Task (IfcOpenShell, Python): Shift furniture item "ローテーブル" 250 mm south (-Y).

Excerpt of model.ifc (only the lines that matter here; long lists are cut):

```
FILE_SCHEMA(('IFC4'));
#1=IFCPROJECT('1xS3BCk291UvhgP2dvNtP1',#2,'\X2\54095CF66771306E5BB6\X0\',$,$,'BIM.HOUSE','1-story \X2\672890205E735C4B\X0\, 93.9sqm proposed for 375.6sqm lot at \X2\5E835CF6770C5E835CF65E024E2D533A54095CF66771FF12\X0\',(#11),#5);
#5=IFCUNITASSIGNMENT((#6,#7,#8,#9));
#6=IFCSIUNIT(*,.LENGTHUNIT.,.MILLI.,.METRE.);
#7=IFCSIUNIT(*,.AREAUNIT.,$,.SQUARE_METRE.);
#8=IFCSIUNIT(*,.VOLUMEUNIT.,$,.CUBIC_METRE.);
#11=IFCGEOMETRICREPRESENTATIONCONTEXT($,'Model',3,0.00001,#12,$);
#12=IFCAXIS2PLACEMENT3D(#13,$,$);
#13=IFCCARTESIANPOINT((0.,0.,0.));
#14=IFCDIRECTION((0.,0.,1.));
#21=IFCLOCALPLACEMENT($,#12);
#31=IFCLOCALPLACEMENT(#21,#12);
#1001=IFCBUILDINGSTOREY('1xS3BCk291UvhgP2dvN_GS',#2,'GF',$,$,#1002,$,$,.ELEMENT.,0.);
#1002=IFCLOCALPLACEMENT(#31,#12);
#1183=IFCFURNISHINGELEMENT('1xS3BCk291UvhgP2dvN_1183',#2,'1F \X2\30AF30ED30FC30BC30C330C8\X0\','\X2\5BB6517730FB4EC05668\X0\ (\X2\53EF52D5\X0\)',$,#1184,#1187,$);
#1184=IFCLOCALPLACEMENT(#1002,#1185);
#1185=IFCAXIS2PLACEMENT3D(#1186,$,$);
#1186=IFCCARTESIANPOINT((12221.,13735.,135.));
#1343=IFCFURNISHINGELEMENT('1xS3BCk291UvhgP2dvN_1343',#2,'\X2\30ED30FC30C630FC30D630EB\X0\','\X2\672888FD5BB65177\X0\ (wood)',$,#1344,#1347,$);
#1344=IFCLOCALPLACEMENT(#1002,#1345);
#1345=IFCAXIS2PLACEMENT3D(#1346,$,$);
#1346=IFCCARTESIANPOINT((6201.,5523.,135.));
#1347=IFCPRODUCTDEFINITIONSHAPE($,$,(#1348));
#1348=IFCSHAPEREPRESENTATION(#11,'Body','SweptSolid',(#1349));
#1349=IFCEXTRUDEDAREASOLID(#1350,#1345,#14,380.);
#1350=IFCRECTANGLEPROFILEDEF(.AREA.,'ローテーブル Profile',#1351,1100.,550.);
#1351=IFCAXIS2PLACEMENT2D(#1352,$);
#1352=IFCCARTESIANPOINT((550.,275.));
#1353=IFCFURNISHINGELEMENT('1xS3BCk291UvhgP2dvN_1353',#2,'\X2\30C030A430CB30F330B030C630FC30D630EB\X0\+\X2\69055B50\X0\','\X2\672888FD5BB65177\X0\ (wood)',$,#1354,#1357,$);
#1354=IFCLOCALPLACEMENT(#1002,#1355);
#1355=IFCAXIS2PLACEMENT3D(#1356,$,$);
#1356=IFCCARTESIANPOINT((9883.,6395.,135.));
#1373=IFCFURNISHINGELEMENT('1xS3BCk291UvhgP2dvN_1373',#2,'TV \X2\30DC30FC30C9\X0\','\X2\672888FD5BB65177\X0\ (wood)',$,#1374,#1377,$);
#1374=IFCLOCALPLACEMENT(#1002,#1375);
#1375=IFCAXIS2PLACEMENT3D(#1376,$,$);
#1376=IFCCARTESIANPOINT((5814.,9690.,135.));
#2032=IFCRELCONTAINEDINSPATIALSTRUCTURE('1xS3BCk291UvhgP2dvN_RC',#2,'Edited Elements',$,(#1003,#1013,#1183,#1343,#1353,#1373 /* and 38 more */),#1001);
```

```python
import ifcopenshell
import ifcopenshell.api.geometry
import ifcopenshell.util.placement

model = ifcopenshell.open("model.ifc")

item = model.by_guid("1xS3BCk291UvhgP2dvN_1343")
matrix = ifcopenshell.util.placement.get_local_placement(item.ObjectPlacement)
matrix[1, 3] -= 250.0
ifcopenshell.api.geometry.edit_object_placement(model, product=item, matrix=matrix, is_si=False)

print(ifcopenshell.util.placement.get_local_placement(item.ObjectPlacement).round(3) + 0.0)

model.write("model_rev.ifc")
```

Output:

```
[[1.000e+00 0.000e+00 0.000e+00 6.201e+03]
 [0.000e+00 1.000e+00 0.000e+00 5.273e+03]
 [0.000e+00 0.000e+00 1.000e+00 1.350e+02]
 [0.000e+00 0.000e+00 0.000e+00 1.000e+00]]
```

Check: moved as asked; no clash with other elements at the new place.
